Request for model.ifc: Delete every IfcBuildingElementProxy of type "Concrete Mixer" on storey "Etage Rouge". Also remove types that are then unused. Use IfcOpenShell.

First a look at what the model holds.

```python
import ifcopenshell
import ifcopenshell.util.element

model = ifcopenshell.open("model.ifc")
print(model.schema)
storey = next(s for s in model.by_type("IfcBuildingStorey") if s.Name == "Etage Rouge")
proxies = [e for e in ifcopenshell.util.element.get_decomposition(storey) if e.is_a("IfcBuildingElementProxy")]
seen = {}
for e in proxies:
    element_type = ifcopenshell.util.element.get_type(e)
    name = element_type.Name if element_type not in (None, e) else None
    seen[name] = seen.get(name, 0) + 1
for name, count in sorted(seen.items(), key=str):
    print(count, "x", name)
```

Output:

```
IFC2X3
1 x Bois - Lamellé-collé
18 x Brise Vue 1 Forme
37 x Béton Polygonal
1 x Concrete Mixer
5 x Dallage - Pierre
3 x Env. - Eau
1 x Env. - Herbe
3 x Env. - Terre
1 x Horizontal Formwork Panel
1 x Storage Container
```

```python
import ifcopenshell
import ifcopenshell.api.root
import ifcopenshell.util.element

model = ifcopenshell.open("model.ifc")

storey = next(s for s in model.by_type("IfcBuildingStorey") if s.Name == "Etage Rouge")
proxies = [e for e in ifcopenshell.util.element.get_decomposition(storey) if e.is_a("IfcBuildingElementProxy")]
targets = [e for e in proxies if (t := ifcopenshell.util.element.get_type(e)) not in (None, e) and t.Name == "Concrete Mixer"]
types = {ifcopenshell.util.element.get_type(e) for e in targets} - {None, *targets}

for e in targets:
    ifcopenshell.api.root.remove_product(model, product=e)
print(len(targets), "removed")

unused = [t for t in types if not ifcopenshell.util.element.get_types(t)]
for t in unused:
    ifcopenshell.api.root.remove_product(model, product=t)
print(len(unused), "unused types removed")

model.write("model_edited.ifc")
```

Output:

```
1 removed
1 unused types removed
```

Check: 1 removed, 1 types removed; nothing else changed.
